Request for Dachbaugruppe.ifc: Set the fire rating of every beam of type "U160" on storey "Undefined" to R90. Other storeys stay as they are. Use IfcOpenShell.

First a look at what the model holds.

```python
import ifcopenshell
import ifcopenshell.util.element

model = ifcopenshell.open("Dachbaugruppe.ifc")
print(model.schema)
storey = next(s for s in model.by_type("IfcBuildingStorey") if s.Name == "Undefined")
beams = [e for e in ifcopenshell.util.element.get_decomposition(storey) if e.is_a("IfcBeam")]
seen = {}
for e in beams:
    element_type = ifcopenshell.util.element.get_type(e)
    key = (element_type.Name if element_type != e and element_type else None, ifcopenshell.util.element.get_pset(e, "Pset_BeamCommon", "FireRating"))
    seen[key] = seen.get(key, 0) + 1
for (name, value), count in sorted(seen.items(), key=str):
    print(count, "x", name, "|", value)
```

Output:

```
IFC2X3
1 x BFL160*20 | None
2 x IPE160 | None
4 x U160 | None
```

```python
import ifcopenshell
import ifcopenshell.api.pset
import ifcopenshell.util.element

model = ifcopenshell.open("Dachbaugruppe.ifc")

storey = next(s for s in model.by_type("IfcBuildingStorey") if s.Name == "Undefined")
beams = [e for e in ifcopenshell.util.element.get_decomposition(storey) if e.is_a("IfcBeam")]

count = 0
for e in beams:
    element_type = ifcopenshell.util.element.get_type(e)
    if element_type in (None, e) or element_type.Name != "U160":
        continue
    # add_pset returns the element's existing set when there is one.
    pset = ifcopenshell.api.pset.add_pset(model, product=e, name="Pset_BeamCommon")
    ifcopenshell.api.pset.edit_pset(model, pset=pset, properties={"FireRating": "R90"})
    count += 1

print(count, "beams updated")

model.write("Dachbaugruppe_v2.ifc")
```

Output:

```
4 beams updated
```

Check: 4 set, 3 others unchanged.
